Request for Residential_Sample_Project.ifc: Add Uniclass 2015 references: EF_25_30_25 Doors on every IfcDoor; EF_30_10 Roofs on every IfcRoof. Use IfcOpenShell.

First a look at what the model holds.

```python
import ifcopenshell

model = ifcopenshell.open("Residential_Sample_Project.ifc")
print(model.schema)
print("classifications:", [c.Name for c in model.by_type("IfcClassification")])
for ifc_class in ("IfcDoor", "IfcRoof", "IfcStair", "IfcWall", "IfcWindow"):
    print(ifc_class, len(model.by_type(ifc_class)))
```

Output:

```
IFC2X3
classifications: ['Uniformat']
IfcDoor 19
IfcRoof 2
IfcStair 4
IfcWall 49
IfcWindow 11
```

```python
import ifcopenshell
import ifcopenshell.api.classification

model = ifcopenshell.open("Residential_Sample_Project.ifc")

# IFC2X3 requires Source and Edition and has no link from the project to the system.
system = model.create_entity("IfcClassification", Source="NBS", Edition="2015", Name="Uniclass 2015")

codes = {
    "IfcDoor": ("EF_25_30_25", "Doors"),
    "IfcRoof": ("EF_30_10", "Roofs"),
}
for ifc_class, (code, name) in codes.items():
    products = model.by_type(ifc_class)
    ifcopenshell.api.classification.add_reference(
        model, products=products, classification=system, identification=code, name=name
    )
    print(code, len(products))

model.write("Residential_Sample_Project-out.ifc")
```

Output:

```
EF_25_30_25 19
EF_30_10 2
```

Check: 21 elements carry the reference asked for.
